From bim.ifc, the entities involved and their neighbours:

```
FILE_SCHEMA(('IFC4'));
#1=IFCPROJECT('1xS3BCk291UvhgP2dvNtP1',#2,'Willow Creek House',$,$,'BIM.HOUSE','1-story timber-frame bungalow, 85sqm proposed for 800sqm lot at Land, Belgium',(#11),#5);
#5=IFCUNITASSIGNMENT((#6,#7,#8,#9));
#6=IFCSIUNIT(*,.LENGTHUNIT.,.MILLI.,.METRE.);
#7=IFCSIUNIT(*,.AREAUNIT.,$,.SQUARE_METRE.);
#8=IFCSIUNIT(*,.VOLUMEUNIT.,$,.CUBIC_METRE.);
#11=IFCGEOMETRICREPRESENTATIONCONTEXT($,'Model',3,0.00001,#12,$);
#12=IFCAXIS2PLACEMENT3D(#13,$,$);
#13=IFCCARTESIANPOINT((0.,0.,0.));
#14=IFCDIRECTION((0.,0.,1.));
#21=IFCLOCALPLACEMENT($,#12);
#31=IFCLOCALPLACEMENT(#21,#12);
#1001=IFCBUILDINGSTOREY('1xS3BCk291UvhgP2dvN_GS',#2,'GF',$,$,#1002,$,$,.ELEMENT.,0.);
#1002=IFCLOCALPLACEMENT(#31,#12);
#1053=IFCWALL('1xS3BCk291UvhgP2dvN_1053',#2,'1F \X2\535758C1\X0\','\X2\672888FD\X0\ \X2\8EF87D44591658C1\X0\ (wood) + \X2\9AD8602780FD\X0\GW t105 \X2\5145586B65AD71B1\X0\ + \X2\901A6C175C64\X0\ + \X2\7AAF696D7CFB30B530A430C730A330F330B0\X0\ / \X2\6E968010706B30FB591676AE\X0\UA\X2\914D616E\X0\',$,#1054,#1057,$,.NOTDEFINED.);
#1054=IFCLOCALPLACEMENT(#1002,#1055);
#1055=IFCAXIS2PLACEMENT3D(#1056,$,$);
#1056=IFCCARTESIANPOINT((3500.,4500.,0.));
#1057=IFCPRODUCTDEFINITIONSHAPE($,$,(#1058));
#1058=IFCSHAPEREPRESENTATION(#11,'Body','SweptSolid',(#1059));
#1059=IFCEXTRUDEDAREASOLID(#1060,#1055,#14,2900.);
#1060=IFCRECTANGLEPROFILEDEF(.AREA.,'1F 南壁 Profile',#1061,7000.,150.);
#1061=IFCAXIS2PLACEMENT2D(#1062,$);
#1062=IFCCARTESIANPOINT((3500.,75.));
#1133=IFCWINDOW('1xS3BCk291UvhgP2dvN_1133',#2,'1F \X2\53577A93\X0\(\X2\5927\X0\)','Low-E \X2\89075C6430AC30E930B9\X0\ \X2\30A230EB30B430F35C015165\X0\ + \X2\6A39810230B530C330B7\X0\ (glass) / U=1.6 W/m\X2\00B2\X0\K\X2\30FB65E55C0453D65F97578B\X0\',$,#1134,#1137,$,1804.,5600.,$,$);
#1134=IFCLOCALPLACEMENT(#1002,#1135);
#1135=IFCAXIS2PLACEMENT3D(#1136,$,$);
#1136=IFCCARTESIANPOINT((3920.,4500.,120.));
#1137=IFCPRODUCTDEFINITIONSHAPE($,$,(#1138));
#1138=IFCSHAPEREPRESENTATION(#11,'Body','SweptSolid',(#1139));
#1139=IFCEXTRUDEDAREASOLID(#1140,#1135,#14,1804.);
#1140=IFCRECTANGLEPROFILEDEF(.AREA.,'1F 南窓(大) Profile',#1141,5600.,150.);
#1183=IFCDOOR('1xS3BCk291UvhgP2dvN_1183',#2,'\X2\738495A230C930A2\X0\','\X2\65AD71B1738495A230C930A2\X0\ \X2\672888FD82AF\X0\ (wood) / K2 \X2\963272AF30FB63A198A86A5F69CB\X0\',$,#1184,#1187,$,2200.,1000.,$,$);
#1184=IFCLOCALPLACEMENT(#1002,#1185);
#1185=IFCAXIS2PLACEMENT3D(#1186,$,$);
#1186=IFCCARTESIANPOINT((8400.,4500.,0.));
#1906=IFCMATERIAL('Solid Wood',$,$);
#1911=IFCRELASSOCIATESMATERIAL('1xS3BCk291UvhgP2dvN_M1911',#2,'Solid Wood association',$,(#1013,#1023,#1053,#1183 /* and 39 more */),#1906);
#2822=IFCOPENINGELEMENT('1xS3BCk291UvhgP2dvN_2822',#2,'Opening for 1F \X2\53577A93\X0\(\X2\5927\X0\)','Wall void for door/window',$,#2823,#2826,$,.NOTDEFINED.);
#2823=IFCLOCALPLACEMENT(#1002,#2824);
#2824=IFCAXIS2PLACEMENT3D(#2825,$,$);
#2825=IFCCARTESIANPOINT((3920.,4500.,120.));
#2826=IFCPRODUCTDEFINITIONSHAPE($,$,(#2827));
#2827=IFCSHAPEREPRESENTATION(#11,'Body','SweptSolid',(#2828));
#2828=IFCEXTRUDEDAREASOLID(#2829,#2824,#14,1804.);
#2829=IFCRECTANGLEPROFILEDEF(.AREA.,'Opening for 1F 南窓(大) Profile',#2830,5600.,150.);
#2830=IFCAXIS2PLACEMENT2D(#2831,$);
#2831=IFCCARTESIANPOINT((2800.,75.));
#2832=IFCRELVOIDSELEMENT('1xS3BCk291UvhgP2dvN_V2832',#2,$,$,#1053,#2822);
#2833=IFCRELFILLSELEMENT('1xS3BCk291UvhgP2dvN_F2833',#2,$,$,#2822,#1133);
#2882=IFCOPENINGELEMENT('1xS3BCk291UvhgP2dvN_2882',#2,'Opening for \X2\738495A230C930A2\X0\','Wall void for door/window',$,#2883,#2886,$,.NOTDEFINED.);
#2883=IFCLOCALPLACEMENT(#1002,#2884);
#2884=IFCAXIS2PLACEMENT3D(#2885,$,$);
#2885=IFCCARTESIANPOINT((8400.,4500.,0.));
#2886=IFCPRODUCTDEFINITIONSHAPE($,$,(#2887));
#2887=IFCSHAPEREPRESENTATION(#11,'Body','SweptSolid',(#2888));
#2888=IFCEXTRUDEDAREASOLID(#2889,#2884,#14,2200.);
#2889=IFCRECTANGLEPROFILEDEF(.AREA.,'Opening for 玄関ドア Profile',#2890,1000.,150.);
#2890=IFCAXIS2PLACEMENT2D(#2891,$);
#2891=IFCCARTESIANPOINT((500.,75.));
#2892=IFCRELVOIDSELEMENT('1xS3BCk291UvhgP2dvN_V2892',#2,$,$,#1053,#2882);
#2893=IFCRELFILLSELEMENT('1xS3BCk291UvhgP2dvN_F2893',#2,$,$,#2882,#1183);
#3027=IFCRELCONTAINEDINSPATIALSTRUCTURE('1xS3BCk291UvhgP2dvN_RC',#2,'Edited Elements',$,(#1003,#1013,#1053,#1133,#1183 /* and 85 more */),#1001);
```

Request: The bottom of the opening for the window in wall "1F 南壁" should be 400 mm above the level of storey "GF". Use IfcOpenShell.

```python
import numpy as np
import ifcopenshell
import ifcopenshell.api.geometry
import ifcopenshell.geom
import ifcopenshell.util.element
import ifcopenshell.util.placement
import ifcopenshell.util.shape
import ifcopenshell.util.unit

model = ifcopenshell.open("bim.ifc")
unit_scale = ifcopenshell.util.unit.calculate_unit_scale(model)

window = model.by_guid("1xS3BCk291UvhgP2dvN_1133")
opening = window.FillsVoids[0].RelatingOpeningElement
storey = ifcopenshell.util.element.get_container(window, ifc_class="IfcBuildingStorey")
level = ifcopenshell.util.placement.get_local_placement(storey.ObjectPlacement)[2, 3]

# The opening's origin need not be at the sill, so measure its lowest point.
shape = ifcopenshell.geom.create_shape(ifcopenshell.geom.settings(), opening)
bottom = ifcopenshell.util.shape.get_shape_bottom_elevation(shape, shape.geometry) / unit_scale
dz = level + 0.4 / unit_scale - bottom

shift = np.array([0.0, 0.0, dz])
# The window is not placed relative to its opening, so move both.
for product in (opening, window):
    matrix = ifcopenshell.util.placement.get_local_placement(product.ObjectPlacement)
    matrix[:3, 3] += shift
    ifcopenshell.api.geometry.edit_object_placement(model, product=product, matrix=matrix, is_si=False)

print(f"moved by {dz * unit_scale:+.3f} m")

model.write("bim_edited.ifc")
```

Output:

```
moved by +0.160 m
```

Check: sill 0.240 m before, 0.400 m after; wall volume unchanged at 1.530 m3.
